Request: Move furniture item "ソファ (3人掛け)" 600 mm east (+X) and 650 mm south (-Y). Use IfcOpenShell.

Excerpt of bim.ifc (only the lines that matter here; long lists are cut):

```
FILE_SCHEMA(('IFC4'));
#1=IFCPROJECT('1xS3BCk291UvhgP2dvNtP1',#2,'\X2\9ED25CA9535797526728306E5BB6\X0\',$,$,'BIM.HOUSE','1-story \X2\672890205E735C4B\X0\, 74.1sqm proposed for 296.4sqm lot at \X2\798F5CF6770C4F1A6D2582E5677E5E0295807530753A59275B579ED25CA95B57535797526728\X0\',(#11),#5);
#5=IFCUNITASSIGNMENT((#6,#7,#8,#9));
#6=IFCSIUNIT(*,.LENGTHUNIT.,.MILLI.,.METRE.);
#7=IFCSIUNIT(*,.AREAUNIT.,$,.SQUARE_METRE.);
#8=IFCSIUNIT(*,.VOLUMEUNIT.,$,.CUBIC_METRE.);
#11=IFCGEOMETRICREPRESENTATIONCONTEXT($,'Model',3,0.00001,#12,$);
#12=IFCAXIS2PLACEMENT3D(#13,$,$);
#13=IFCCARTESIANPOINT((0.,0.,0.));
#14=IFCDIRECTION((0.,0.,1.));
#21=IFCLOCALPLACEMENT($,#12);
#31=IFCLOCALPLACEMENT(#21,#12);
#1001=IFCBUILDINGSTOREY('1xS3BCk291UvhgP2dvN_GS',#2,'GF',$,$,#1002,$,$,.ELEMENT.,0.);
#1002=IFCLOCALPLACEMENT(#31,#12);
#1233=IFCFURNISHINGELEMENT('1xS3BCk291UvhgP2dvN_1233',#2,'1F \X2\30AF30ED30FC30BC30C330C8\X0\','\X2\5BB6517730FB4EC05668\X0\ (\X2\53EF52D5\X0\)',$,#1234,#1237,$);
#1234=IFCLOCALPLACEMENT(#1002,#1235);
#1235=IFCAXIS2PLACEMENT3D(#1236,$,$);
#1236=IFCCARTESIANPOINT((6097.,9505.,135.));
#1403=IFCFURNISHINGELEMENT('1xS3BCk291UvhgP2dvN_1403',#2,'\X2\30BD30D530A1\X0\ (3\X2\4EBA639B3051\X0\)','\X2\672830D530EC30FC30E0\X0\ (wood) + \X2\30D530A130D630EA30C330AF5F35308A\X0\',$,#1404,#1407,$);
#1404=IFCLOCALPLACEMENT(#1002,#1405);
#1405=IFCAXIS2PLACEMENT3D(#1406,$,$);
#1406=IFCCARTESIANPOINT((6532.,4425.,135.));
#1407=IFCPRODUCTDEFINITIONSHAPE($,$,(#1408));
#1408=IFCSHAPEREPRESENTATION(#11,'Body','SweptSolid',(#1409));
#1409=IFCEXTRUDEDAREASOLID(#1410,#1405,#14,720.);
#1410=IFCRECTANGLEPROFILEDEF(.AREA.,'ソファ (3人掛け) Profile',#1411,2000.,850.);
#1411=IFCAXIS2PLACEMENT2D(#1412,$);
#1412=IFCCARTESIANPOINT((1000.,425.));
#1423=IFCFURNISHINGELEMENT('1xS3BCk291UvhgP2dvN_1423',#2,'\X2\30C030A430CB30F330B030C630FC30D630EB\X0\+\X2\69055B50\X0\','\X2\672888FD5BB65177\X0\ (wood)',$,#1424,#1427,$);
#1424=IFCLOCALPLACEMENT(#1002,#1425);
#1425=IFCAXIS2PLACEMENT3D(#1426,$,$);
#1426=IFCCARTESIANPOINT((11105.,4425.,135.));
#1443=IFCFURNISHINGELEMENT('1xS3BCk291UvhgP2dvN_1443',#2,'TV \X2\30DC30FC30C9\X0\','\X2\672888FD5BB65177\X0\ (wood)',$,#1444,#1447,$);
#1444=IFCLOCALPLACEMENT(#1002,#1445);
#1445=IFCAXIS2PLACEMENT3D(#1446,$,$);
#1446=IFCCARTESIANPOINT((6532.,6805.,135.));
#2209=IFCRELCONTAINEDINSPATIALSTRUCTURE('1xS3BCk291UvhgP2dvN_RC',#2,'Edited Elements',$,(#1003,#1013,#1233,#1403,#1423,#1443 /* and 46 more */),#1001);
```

```python
import ifcopenshell
import ifcopenshell.api.geometry
import ifcopenshell.util.placement

model = ifcopenshell.open("bim.ifc")

item = model.by_id(1403)
matrix = ifcopenshell.util.placement.get_local_placement(item.ObjectPlacement)
matrix[0, 3] += 600.0
matrix[1, 3] -= 650.0
ifcopenshell.api.geometry.edit_object_placement(model, product=item, matrix=matrix, is_si=False)

print(ifcopenshell.util.placement.get_local_placement(item.ObjectPlacement).round(3) + 0.0)

model.write("bim_edited.ifc")
```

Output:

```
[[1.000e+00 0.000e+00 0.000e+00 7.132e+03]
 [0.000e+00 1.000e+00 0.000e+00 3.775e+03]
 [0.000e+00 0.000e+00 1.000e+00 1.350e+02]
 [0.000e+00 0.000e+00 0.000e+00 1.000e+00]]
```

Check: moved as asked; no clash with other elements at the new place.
